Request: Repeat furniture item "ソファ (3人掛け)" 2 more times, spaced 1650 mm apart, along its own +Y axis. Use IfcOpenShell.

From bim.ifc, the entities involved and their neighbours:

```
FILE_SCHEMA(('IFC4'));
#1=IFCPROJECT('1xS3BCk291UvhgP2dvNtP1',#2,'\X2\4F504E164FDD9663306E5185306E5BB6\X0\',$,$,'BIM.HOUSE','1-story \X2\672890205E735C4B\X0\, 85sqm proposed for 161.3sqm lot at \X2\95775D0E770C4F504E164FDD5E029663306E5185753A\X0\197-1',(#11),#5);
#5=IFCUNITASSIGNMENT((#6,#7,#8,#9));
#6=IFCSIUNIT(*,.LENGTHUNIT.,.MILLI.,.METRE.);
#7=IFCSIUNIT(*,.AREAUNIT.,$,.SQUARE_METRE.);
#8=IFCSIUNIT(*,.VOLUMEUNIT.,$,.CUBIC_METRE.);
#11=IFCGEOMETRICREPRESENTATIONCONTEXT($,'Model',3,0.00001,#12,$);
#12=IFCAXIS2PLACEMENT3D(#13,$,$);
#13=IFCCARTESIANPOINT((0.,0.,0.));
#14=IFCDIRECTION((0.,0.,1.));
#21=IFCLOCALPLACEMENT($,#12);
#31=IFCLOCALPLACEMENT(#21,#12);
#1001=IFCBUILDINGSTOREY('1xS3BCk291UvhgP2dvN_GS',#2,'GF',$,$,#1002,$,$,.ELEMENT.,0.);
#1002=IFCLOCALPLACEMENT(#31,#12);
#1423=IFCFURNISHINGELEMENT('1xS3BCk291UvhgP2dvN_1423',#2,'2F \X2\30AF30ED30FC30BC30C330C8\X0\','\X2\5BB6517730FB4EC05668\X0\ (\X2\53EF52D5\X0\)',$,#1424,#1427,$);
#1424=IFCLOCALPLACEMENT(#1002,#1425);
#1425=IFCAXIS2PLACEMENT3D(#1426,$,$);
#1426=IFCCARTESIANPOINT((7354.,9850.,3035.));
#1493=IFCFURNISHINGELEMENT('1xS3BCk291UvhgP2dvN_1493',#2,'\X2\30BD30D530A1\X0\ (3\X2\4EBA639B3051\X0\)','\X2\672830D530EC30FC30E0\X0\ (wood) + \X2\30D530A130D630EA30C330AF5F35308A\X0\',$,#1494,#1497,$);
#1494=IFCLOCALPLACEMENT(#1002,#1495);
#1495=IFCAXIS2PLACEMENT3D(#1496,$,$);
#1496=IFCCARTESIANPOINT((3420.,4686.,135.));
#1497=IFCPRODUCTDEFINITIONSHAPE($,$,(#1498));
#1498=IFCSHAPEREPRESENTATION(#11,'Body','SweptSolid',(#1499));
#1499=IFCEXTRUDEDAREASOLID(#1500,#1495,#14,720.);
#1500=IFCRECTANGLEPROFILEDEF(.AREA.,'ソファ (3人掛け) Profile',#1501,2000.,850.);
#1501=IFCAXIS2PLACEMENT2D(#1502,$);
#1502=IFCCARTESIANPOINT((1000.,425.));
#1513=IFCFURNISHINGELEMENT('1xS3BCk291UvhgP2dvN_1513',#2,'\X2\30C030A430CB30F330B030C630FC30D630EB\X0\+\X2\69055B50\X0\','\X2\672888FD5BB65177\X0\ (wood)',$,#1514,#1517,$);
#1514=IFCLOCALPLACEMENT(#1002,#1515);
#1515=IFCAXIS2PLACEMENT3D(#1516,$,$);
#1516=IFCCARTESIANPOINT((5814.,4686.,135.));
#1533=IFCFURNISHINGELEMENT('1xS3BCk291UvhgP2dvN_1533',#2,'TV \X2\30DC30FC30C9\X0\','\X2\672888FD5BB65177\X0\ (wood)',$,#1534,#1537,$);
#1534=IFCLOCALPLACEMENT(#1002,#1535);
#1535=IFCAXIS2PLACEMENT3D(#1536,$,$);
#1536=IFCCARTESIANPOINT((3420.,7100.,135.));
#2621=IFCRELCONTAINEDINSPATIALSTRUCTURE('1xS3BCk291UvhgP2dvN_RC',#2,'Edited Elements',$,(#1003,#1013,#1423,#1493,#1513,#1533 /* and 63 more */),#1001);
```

```python
import ifcopenshell
import ifcopenshell.api.geometry
import ifcopenshell.api.root
import ifcopenshell.util.element
import ifcopenshell.util.placement
import ifcopenshell.util.unit

model = ifcopenshell.open("bim.ifc")
unit_scale = ifcopenshell.util.unit.calculate_unit_scale(model)


def reuse_history(source, copy):
    """copy_class also copies each property set's owner history, people and application; keep the originals."""
    for rel in copy.IsDefinedBy:
        if rel.is_a("IfcRelDefinesByProperties") and (history := rel.RelatingPropertyDefinition.OwnerHistory):
            rel.RelatingPropertyDefinition.OwnerHistory = source.OwnerHistory
            ifcopenshell.util.element.remove_deep2(model, history)


source = model.by_guid("1xS3BCk291UvhgP2dvN_1493")
base = ifcopenshell.util.placement.get_local_placement(source.ObjectPlacement)
step = base[:3, 1] * 1.65 / unit_scale

for i in range(1, 3):
    copy = ifcopenshell.api.root.copy_class(model, product=source)
    copy.Representation = ifcopenshell.util.element.copy_deep(
        model, source.Representation, exclude=["IfcGeometricRepresentationContext", "IfcRepresentationMap"]
    )
    reuse_history(source, copy)
    matrix = base.copy()
    matrix[:3, 3] += i * step
    print("added at", matrix[:3, 3].round(3) + 0.0)
    ifcopenshell.api.geometry.edit_object_placement(model, product=copy, matrix=matrix, is_si=False)

model.write("bim_v2.ifc")
```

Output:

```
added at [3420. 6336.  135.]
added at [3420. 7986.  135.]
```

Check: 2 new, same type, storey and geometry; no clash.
